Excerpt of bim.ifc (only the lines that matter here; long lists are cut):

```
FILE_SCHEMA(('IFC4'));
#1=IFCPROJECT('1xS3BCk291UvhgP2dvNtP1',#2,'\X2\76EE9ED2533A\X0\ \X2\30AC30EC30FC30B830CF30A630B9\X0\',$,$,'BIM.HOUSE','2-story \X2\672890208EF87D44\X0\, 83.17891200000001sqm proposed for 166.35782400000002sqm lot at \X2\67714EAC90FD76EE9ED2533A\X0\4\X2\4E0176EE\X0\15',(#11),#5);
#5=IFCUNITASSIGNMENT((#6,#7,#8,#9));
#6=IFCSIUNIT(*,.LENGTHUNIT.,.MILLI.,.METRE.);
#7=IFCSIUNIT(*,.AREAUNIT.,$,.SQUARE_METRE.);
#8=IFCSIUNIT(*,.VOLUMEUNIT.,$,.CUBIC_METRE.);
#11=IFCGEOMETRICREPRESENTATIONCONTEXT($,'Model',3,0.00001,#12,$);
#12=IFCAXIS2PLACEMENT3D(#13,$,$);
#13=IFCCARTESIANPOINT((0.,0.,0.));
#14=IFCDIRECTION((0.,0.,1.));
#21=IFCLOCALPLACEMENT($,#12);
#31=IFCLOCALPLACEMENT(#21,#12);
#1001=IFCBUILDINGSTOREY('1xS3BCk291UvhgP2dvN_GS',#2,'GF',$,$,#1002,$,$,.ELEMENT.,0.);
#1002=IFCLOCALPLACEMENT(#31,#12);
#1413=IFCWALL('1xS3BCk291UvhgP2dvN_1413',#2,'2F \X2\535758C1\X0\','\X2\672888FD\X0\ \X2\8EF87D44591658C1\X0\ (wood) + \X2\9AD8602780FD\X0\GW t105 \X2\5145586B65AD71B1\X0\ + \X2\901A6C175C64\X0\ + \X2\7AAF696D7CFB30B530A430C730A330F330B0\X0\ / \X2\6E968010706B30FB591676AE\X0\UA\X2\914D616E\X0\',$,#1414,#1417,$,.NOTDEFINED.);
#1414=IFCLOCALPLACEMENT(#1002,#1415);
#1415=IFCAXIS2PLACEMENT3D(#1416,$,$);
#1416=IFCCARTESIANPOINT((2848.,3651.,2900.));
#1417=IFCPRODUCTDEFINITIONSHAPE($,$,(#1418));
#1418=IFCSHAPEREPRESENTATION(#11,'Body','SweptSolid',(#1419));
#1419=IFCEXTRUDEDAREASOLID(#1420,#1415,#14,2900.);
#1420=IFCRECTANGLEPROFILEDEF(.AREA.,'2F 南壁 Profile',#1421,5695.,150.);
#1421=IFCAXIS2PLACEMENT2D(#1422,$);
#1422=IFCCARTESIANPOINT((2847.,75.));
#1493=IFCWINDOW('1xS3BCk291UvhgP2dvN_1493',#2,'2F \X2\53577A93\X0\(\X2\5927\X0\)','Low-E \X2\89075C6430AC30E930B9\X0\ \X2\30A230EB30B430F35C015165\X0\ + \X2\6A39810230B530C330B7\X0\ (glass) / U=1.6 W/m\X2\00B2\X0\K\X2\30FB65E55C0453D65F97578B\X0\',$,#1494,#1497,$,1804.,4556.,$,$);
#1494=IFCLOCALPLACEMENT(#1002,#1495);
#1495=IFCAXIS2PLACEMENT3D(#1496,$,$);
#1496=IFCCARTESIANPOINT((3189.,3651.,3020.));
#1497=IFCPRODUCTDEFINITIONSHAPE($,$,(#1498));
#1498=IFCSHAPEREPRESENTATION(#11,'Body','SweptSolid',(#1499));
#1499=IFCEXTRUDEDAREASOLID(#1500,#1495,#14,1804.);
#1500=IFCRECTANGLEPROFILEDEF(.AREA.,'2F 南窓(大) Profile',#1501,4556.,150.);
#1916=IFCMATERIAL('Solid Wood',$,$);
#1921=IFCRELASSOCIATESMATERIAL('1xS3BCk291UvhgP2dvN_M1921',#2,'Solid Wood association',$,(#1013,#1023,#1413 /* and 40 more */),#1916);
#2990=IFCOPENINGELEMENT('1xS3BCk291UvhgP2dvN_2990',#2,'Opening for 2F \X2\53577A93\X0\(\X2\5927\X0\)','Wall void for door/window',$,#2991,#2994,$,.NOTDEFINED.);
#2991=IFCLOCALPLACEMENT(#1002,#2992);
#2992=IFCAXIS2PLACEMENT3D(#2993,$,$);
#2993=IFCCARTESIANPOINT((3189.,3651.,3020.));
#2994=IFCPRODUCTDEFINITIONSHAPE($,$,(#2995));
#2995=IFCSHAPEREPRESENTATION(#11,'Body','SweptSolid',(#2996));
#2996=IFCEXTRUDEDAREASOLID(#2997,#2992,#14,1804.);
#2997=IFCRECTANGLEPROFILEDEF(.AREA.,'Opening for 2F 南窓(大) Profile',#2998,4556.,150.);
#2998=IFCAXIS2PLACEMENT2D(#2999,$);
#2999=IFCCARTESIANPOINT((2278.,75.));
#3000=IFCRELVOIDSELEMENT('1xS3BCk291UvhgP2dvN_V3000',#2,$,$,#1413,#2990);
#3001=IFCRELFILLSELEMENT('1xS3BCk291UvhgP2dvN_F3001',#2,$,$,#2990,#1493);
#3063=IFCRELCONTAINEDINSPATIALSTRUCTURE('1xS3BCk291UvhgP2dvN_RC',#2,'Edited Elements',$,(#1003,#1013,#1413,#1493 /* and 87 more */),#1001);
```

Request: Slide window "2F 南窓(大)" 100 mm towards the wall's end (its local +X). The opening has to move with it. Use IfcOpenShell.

```python
import ifcopenshell
import ifcopenshell.api.geometry
import ifcopenshell.util.placement

model = ifcopenshell.open("bim.ifc")

window = model.by_guid("1xS3BCk291UvhgP2dvN_1493")
opening = window.FillsVoids[0].RelatingOpeningElement
wall = opening.VoidsElements[0].RelatingBuildingElement

wall_matrix = ifcopenshell.util.placement.get_local_placement(wall.ObjectPlacement)
shift = wall_matrix[:3, 0] * 100.0
before = ifcopenshell.util.placement.get_local_placement(window.ObjectPlacement)[:3, 3].copy()

# The window is not placed relative to its opening, so move both.
for product in (opening, window):
    matrix = ifcopenshell.util.placement.get_local_placement(product.ObjectPlacement)
    matrix[:3, 3] += shift
    ifcopenshell.api.geometry.edit_object_placement(model, product=product, matrix=matrix, is_si=False)

after = ifcopenshell.util.placement.get_local_placement(window.ObjectPlacement)[:3, 3]
print("window moved by", (after - before).round(3) + 0.0)

model.write("bim_rev.ifc")
```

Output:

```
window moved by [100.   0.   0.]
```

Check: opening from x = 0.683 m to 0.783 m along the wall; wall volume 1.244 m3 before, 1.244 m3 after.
